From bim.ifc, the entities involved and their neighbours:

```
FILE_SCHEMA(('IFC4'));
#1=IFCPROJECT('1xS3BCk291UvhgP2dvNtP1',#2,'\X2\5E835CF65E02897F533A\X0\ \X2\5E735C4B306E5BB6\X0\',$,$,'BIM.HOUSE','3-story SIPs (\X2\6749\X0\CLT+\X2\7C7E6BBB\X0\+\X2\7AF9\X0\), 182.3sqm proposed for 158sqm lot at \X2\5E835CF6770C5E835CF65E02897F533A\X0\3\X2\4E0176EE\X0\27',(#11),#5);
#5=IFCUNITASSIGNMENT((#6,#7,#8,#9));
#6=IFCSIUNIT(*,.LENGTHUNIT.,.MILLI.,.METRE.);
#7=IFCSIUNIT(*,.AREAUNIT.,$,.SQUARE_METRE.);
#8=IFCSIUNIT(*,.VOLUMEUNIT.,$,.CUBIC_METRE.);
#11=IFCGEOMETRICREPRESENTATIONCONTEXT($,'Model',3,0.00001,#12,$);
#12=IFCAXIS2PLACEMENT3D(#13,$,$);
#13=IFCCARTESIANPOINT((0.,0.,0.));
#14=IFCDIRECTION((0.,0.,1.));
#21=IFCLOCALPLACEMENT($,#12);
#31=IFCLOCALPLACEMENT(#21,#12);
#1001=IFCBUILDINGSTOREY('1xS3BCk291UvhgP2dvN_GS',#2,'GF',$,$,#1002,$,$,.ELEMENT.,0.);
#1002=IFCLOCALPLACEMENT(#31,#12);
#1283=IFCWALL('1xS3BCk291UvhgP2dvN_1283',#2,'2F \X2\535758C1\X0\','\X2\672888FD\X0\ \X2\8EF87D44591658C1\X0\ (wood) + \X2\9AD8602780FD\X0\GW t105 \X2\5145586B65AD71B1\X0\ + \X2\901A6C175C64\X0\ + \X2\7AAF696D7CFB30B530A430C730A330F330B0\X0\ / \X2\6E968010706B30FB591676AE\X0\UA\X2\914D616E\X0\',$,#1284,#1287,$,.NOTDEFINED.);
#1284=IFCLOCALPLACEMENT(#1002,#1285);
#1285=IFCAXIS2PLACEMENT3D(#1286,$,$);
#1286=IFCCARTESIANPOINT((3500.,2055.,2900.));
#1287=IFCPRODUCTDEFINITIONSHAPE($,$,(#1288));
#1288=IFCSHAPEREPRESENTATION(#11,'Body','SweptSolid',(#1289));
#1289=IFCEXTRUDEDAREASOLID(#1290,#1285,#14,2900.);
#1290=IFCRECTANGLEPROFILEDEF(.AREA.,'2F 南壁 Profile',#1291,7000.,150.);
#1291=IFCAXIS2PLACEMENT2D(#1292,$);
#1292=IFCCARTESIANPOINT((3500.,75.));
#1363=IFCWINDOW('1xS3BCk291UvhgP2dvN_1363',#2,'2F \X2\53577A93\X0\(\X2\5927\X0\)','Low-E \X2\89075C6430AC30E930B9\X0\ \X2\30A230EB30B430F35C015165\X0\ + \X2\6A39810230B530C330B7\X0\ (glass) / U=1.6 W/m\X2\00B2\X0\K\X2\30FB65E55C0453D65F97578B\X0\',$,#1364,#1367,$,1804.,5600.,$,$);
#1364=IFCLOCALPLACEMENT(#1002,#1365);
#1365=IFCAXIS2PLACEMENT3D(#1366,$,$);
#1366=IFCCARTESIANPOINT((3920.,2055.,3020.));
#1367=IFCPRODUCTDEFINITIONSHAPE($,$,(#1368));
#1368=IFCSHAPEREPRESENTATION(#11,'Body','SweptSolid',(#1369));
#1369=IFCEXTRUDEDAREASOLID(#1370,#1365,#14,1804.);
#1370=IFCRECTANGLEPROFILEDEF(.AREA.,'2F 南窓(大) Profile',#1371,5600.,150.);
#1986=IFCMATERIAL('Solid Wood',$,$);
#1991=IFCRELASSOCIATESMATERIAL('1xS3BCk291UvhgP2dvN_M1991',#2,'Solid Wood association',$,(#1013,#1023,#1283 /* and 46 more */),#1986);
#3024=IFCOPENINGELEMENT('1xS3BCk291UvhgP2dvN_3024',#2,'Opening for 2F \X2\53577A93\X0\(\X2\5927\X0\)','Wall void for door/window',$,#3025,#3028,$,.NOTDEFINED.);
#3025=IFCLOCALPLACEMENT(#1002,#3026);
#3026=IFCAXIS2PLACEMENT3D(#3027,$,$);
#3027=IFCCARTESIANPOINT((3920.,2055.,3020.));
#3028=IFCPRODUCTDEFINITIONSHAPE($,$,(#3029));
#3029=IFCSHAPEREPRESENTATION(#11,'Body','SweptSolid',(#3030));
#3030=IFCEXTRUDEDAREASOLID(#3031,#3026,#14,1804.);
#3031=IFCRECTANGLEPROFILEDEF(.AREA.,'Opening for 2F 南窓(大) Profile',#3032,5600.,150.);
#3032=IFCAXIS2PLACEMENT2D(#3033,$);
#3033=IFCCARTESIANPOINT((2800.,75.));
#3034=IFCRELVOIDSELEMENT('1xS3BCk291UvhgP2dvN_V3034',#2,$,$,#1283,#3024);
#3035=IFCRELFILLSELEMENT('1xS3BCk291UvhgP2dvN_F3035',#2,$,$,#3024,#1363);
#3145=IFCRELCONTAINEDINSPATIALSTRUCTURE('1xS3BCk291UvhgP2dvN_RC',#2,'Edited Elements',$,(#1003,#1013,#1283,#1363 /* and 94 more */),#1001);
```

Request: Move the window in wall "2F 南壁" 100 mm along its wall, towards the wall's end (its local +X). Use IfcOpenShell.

```python
import ifcopenshell
import ifcopenshell.api.geometry
import ifcopenshell.util.placement
import ifcopenshell.util.unit

model = ifcopenshell.open("bim.ifc")
unit_scale = ifcopenshell.util.unit.calculate_unit_scale(model)

window = model.by_guid("1xS3BCk291UvhgP2dvN_1363")
opening = window.FillsVoids[0].RelatingOpeningElement
wall = opening.VoidsElements[0].RelatingBuildingElement

wall_matrix = ifcopenshell.util.placement.get_local_placement(wall.ObjectPlacement)
shift = wall_matrix[:3, 0] * 0.1 / unit_scale
before = ifcopenshell.util.placement.get_local_placement(window.ObjectPlacement)[:3, 3].copy()

# The window is not placed relative to its opening, so move both.
for product in (opening, window):
    matrix = ifcopenshell.util.placement.get_local_placement(product.ObjectPlacement)
    matrix[:3, 3] += shift
    ifcopenshell.api.geometry.edit_object_placement(model, product=product, matrix=matrix, is_si=False)

after = ifcopenshell.util.placement.get_local_placement(window.ObjectPlacement)[:3, 3]
print("window moved by", (after - before).round(3) + 0.0)

model.write("bim-out.ifc")
```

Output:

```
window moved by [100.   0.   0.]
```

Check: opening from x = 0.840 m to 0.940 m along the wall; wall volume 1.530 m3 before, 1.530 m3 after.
